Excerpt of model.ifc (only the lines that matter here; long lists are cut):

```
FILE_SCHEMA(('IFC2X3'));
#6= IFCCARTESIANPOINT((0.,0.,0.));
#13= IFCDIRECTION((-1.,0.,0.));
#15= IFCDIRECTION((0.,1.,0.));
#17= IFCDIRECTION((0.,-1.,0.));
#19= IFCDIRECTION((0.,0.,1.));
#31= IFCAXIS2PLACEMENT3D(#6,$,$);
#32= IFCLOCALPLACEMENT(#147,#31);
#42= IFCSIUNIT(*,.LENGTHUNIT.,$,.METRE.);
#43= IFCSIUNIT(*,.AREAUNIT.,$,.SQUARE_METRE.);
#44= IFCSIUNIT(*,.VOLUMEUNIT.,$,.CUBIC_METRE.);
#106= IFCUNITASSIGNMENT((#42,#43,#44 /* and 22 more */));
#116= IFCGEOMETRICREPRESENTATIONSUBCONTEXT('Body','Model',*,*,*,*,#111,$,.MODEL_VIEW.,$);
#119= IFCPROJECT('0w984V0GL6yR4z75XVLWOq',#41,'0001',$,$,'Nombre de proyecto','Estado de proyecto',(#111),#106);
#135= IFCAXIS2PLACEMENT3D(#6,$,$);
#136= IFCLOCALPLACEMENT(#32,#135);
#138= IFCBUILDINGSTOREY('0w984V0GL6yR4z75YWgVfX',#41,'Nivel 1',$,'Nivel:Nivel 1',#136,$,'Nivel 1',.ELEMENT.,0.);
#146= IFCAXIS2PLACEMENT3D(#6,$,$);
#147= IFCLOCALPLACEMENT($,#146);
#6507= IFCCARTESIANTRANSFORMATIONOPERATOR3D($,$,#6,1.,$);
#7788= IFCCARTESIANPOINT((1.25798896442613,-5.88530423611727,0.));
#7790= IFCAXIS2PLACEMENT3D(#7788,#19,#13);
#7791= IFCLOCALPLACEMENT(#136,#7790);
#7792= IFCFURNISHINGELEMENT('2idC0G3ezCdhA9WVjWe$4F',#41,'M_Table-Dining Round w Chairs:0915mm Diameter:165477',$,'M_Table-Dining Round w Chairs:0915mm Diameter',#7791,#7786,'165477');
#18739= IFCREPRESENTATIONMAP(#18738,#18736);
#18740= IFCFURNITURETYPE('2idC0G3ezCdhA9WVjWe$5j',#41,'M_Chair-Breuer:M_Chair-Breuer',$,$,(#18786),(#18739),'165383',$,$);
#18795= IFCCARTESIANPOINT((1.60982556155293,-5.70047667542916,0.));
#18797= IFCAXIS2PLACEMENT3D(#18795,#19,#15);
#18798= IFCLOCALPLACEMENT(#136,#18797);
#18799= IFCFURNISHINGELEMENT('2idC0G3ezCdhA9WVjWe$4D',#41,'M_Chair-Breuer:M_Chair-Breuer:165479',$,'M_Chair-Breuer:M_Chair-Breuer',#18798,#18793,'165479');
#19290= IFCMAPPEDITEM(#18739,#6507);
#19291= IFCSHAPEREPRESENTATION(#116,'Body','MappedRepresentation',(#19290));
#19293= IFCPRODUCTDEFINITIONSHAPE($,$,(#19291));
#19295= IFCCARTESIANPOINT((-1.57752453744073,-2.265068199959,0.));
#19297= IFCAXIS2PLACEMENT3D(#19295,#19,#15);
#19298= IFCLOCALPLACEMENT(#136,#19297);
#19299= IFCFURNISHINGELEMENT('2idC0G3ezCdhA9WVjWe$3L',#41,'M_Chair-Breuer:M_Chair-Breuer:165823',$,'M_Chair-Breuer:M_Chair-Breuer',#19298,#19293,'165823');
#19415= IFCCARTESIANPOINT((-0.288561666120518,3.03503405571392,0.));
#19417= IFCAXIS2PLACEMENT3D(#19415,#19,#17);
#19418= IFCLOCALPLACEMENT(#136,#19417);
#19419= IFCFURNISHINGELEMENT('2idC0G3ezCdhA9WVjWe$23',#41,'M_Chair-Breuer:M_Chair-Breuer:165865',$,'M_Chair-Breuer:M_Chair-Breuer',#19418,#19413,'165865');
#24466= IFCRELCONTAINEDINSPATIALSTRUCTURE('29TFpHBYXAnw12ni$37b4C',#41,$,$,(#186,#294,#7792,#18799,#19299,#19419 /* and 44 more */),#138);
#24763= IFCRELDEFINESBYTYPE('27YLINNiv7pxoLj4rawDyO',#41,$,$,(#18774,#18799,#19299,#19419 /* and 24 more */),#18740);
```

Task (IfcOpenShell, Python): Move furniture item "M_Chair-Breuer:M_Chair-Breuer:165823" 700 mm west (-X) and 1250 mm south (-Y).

```python
import ifcopenshell
import ifcopenshell.api.geometry
import ifcopenshell.util.placement
import ifcopenshell.util.unit

model = ifcopenshell.open("model.ifc")
unit_scale = ifcopenshell.util.unit.calculate_unit_scale(model)

item = model.by_guid("2idC0G3ezCdhA9WVjWe$3L")
matrix = ifcopenshell.util.placement.get_local_placement(item.ObjectPlacement)
matrix[0, 3] -= 0.7 / unit_scale
matrix[1, 3] -= 1.25 / unit_scale
ifcopenshell.api.geometry.edit_object_placement(model, product=item, matrix=matrix, is_si=False)

print(ifcopenshell.util.placement.get_local_placement(item.ObjectPlacement).round(3) + 0.0)

model.write("model_rev.ifc")
```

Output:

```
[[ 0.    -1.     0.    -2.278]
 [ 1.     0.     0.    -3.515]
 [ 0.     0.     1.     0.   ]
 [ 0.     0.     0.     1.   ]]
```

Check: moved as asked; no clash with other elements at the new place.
